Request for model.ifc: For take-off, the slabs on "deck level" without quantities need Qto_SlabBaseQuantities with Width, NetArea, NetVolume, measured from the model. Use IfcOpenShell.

First a look at what the model holds.

```python
import ifcopenshell
import ifcopenshell.util.element
import ifcopenshell.util.unit

model = ifcopenshell.open("model.ifc")
print(model.schema)
for unit_type in ("LENGTHUNIT", "AREAUNIT", "VOLUMEUNIT"):
    print(unit_type, ifcopenshell.util.unit.calculate_unit_scale(model, unit_type))
storey = next(s for s in model.by_type("IfcBuildingStorey") if s.Name == "deck level")
slabs = [e for e in ifcopenshell.util.element.get_decomposition(storey) if e.is_a("IfcSlab")]
for e in sorted(slabs, key=lambda e: e.id()):
    print(e.id(), e.is_a(), e.Name, list(ifcopenshell.util.element.get_psets(e, qtos_only=True)), sep=" | ")
```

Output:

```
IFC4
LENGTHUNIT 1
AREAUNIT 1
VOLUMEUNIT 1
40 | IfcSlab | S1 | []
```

```python
import ifcopenshell
import ifcopenshell.api.pset
import ifcopenshell.geom
import ifcopenshell.util.element
import ifcopenshell.util.shape
import ifcopenshell.util.unit

model = ifcopenshell.open("model.ifc")
unit_scale = ifcopenshell.util.unit.calculate_unit_scale(model)
area_scale = ifcopenshell.util.unit.calculate_unit_scale(model, "AREAUNIT")
volume_scale = ifcopenshell.util.unit.calculate_unit_scale(model, "VOLUMEUNIT")
settings = ifcopenshell.geom.settings()

storey = next(s for s in model.by_type("IfcBuildingStorey") if s.Name == "deck level")
slabs = [e for e in ifcopenshell.util.element.get_decomposition(storey) if e.is_a("IfcSlab")]

for e in sorted(slabs, key=lambda e: e.id()):
    if ifcopenshell.util.element.get_psets(e, qtos_only=True, should_inherit=False):
        continue
    # Geometry comes back in metres, in the element's own axes.
    shape = ifcopenshell.geom.create_shape(settings, e)
    values = {
        "Width": ifcopenshell.util.shape.get_z(shape.geometry) / unit_scale,
        "NetArea": ifcopenshell.util.shape.get_footprint_area(shape.geometry) / area_scale,
        "NetVolume": ifcopenshell.util.shape.get_volume(shape.geometry) / volume_scale,
    }
    qto = ifcopenshell.api.pset.add_qto(model, product=e, name="Qto_SlabBaseQuantities")
    ifcopenshell.api.pset.edit_qto(model, qto=qto, properties=values)
    print(e.id(), {k: round(v, 3) for k, v in values.items()})

model.write("model_edited.ifc")
```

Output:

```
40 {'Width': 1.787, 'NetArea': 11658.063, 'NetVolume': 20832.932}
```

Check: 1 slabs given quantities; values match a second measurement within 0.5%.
